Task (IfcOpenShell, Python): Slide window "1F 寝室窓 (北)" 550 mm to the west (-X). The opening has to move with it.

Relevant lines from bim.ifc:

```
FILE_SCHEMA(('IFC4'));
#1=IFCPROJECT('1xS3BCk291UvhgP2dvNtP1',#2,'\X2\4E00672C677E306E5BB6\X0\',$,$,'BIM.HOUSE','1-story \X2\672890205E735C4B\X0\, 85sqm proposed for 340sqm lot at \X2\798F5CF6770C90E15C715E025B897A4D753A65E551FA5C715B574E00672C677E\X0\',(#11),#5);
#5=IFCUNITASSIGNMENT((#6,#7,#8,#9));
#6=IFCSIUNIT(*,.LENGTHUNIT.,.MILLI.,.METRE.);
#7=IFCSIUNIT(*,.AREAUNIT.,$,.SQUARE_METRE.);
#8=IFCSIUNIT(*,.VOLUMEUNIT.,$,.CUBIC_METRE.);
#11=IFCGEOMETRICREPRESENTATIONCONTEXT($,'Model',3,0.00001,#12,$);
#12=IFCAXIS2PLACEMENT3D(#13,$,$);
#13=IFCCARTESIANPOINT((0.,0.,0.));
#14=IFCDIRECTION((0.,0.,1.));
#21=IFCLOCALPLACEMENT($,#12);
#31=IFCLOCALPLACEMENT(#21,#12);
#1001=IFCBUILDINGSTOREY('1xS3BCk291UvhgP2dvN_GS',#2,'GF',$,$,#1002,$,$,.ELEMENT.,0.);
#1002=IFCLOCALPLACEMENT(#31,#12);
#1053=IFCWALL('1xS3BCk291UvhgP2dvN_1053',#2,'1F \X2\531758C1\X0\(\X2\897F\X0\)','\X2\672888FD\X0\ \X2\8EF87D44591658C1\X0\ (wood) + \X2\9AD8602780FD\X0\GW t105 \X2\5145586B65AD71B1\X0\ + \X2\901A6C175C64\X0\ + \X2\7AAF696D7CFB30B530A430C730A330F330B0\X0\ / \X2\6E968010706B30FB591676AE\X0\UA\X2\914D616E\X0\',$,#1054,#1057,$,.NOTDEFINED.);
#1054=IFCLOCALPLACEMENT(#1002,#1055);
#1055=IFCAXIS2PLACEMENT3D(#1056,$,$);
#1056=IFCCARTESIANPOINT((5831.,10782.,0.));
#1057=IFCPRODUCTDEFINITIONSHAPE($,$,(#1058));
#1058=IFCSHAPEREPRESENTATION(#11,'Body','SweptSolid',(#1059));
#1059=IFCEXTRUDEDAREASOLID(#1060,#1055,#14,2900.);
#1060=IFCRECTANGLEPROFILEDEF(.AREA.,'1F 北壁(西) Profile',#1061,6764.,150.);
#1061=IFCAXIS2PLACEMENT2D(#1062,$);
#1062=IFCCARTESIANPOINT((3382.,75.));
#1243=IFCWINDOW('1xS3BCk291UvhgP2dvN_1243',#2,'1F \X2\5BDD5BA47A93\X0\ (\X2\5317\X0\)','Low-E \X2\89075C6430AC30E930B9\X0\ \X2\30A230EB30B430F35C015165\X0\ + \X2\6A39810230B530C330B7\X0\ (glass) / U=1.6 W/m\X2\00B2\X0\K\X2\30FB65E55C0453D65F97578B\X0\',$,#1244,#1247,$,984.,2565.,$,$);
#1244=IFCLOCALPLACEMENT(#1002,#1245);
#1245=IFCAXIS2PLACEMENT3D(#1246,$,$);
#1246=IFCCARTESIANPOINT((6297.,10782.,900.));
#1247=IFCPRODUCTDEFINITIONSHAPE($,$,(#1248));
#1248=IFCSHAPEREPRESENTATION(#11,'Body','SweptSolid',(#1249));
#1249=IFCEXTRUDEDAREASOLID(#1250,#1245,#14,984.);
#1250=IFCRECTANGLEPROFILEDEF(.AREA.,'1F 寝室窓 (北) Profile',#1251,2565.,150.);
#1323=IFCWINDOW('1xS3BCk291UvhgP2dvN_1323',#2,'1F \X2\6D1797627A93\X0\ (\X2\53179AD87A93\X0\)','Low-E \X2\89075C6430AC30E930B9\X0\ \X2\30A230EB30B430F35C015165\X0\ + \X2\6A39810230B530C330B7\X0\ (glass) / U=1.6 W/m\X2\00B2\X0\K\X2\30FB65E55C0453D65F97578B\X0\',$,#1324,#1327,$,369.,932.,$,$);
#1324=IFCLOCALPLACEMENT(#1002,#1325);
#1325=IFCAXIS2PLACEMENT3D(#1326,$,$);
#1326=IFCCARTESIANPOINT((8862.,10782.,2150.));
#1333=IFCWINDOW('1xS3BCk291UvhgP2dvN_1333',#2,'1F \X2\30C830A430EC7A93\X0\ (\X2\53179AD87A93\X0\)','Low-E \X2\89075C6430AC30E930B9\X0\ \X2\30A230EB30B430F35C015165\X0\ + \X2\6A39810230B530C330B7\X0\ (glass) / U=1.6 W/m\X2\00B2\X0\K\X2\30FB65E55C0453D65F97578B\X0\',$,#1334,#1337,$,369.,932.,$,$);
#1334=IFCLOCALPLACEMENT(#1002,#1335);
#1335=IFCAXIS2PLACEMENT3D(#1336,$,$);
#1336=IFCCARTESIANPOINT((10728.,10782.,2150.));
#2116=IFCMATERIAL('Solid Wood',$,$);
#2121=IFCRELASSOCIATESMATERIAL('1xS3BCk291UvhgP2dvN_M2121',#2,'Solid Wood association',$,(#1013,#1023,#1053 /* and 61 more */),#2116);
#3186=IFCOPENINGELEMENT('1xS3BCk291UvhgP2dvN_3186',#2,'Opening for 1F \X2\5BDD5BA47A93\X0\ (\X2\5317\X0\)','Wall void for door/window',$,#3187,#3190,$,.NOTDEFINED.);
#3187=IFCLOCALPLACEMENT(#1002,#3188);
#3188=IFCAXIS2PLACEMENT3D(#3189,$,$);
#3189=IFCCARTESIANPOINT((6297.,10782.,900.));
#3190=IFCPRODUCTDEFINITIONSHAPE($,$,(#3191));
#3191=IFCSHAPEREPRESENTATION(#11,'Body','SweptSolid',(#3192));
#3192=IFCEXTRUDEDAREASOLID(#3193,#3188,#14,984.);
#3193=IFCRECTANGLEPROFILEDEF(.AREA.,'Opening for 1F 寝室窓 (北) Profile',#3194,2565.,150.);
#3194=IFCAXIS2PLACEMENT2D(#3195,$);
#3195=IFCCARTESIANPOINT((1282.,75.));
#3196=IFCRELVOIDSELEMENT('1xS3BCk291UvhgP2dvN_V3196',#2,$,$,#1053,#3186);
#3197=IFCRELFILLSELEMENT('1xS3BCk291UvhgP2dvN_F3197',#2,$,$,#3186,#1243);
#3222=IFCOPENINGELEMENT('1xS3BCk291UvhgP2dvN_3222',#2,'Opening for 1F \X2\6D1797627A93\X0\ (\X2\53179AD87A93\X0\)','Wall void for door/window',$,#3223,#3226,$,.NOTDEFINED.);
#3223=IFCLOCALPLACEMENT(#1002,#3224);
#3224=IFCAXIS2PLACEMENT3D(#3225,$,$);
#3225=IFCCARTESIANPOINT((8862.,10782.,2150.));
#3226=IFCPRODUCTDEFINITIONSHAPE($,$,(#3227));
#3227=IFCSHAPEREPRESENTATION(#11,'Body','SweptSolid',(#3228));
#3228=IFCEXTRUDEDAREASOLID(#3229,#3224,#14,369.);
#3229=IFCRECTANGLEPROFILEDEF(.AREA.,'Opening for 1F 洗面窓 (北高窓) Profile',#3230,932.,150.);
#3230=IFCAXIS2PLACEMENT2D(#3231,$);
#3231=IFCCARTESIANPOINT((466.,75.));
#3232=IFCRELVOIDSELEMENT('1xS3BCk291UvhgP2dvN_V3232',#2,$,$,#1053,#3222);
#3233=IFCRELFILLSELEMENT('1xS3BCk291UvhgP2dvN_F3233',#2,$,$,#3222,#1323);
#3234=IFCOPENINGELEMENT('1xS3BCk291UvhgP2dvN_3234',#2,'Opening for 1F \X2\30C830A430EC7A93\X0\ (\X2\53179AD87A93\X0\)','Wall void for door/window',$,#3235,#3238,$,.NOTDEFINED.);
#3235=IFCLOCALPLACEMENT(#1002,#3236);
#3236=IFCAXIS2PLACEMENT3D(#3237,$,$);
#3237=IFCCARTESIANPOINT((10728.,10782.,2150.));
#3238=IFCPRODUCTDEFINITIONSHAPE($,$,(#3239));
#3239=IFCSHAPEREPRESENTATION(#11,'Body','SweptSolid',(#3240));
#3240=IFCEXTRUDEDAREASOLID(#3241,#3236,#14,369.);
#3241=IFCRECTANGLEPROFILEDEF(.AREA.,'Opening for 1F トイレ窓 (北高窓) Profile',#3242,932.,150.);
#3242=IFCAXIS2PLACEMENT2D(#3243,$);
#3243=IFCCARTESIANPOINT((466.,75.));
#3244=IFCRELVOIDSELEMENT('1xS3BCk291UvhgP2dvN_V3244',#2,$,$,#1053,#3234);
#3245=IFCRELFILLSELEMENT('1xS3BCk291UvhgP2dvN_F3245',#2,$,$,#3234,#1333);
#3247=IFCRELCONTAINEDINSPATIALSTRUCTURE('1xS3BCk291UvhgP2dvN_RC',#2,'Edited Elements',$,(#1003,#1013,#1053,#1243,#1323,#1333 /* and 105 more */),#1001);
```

```python
import ifcopenshell
import ifcopenshell.api.geometry
import ifcopenshell.util.placement
import ifcopenshell.util.unit

model = ifcopenshell.open("bim.ifc")
unit_scale = ifcopenshell.util.unit.calculate_unit_scale(model)

window = model.by_guid("1xS3BCk291UvhgP2dvN_1243")
opening = window.FillsVoids[0].RelatingOpeningElement
wall = opening.VoidsElements[0].RelatingBuildingElement

wall_matrix = ifcopenshell.util.placement.get_local_placement(wall.ObjectPlacement)
shift = wall_matrix[:3, 0] * -0.55 / unit_scale
before = ifcopenshell.util.placement.get_local_placement(window.ObjectPlacement)[:3, 3].copy()

# The window is not placed relative to its opening, so move both.
for product in (opening, window):
    matrix = ifcopenshell.util.placement.get_local_placement(product.ObjectPlacement)
    matrix[:3, 3] += shift
    ifcopenshell.api.geometry.edit_object_placement(model, product=product, matrix=matrix, is_si=False)

after = ifcopenshell.util.placement.get_local_placement(window.ObjectPlacement)[:3, 3]
print("window moved by", (after - before).round(3) + 0.0)

model.write("bim_edited.ifc")
```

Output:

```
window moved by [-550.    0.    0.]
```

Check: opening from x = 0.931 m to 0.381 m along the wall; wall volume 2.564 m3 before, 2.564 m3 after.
